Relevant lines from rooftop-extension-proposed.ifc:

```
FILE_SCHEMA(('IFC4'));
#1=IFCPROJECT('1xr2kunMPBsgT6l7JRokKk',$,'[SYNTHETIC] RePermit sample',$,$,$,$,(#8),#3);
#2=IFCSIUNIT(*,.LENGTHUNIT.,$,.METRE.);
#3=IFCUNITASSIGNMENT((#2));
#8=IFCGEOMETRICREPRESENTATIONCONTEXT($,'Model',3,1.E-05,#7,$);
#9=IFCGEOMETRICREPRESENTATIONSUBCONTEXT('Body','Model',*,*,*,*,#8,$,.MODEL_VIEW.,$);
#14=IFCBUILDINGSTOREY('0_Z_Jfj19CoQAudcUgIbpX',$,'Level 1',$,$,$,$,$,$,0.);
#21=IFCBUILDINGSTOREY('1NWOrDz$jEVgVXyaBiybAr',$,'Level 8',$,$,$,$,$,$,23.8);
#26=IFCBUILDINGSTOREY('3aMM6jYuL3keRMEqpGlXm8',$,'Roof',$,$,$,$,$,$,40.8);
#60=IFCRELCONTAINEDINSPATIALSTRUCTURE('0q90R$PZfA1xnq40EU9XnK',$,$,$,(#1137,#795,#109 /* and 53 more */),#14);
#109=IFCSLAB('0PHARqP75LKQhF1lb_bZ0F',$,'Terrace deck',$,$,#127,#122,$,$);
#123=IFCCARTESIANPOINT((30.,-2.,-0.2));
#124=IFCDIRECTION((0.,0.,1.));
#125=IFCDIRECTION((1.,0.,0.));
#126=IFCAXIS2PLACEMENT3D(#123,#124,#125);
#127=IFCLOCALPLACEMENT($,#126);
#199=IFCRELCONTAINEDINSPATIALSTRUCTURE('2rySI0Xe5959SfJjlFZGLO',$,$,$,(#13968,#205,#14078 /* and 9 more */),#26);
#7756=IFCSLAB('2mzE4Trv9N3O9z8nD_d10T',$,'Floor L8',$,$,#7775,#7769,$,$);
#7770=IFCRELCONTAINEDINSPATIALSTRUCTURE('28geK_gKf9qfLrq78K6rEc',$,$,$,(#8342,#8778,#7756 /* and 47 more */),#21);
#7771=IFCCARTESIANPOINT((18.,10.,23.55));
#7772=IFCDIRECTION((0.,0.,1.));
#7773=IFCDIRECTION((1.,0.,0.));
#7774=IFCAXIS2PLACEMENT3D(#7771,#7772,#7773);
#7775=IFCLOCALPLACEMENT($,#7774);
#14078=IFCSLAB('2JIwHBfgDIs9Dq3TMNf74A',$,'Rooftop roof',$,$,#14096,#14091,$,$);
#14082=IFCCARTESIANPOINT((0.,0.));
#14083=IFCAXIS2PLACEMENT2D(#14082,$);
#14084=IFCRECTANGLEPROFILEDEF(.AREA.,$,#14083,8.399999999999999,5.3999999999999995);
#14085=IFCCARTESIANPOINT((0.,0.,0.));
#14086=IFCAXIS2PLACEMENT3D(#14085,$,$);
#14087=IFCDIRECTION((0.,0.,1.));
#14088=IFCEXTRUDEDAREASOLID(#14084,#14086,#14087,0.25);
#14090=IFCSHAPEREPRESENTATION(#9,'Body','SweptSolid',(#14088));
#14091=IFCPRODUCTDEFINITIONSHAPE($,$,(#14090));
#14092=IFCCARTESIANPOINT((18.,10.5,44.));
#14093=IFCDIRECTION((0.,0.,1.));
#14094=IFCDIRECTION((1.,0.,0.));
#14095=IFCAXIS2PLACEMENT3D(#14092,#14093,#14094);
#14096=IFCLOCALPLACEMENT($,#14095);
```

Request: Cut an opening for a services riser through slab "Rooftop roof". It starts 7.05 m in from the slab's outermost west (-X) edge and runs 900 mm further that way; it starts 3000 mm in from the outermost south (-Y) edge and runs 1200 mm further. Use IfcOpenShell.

```python
import numpy as np
import ifcopenshell
import ifcopenshell.api.feature
import ifcopenshell.api.geometry
import ifcopenshell.api.root
import ifcopenshell.geom
import ifcopenshell.util.placement
import ifcopenshell.util.representation
import ifcopenshell.util.shape
import ifcopenshell.util.unit

model = ifcopenshell.open("rooftop-extension-proposed.ifc")
unit_scale = ifcopenshell.util.unit.calculate_unit_scale(model)
settings = ifcopenshell.geom.settings()


def volume(element):
    """Net volume in cubic metres, openings subtracted."""
    shape = ifcopenshell.geom.create_shape(settings, element)
    return ifcopenshell.util.shape.get_volume(shape.geometry)


slab = model.by_guid("2JIwHBfgDIs9Dq3TMNf74A")
before = volume(slab)

# Extent in the slab's own axes, in metres. The edges named are its -X and -Y sides.
slab_shape = ifcopenshell.geom.create_shape(settings, slab)
vertices = ifcopenshell.util.shape.get_vertices(slab_shape.geometry)
x_min, y_min, bottom = vertices.min(axis=0)
top = vertices[:, 2].max()

opening = ifcopenshell.api.root.create_entity(model, ifc_class="IfcOpeningElement", name="Services riser opening", predefined_type="OPENING")
context = ifcopenshell.util.representation.get_context(model, "Model", "Body", "MODEL_VIEW")
width, depth = 0.9, 1.2
outline = [(0.0, 0.0), (width, 0.0), (width, depth), (0.0, depth), (0.0, 0.0)]
# Overshoot both faces by 50 mm so the cut is clean.
shape = ifcopenshell.api.geometry.add_slab_representation(
    model, context=context, depth=top - bottom + 0.1, polyline=outline
)
ifcopenshell.api.geometry.assign_representation(model, product=opening, representation=shape)

matrix = ifcopenshell.util.placement.get_local_placement(slab.ObjectPlacement)
matrix[:, 3] = matrix @ np.append(np.array([x_min + 7.05, y_min + 3, bottom - 0.05]) / unit_scale, 1.0)
ifcopenshell.api.geometry.edit_object_placement(model, product=opening, matrix=matrix, is_si=False)
ifcopenshell.api.feature.add_feature(model, feature=opening, element=slab)

after = volume(slab)

print(f"slab volume {before:.3f} -> {after:.3f} m3")

model.write("rooftop-extension-proposed-out.ifc")
```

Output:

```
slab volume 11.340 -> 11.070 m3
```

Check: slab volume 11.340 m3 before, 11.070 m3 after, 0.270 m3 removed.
